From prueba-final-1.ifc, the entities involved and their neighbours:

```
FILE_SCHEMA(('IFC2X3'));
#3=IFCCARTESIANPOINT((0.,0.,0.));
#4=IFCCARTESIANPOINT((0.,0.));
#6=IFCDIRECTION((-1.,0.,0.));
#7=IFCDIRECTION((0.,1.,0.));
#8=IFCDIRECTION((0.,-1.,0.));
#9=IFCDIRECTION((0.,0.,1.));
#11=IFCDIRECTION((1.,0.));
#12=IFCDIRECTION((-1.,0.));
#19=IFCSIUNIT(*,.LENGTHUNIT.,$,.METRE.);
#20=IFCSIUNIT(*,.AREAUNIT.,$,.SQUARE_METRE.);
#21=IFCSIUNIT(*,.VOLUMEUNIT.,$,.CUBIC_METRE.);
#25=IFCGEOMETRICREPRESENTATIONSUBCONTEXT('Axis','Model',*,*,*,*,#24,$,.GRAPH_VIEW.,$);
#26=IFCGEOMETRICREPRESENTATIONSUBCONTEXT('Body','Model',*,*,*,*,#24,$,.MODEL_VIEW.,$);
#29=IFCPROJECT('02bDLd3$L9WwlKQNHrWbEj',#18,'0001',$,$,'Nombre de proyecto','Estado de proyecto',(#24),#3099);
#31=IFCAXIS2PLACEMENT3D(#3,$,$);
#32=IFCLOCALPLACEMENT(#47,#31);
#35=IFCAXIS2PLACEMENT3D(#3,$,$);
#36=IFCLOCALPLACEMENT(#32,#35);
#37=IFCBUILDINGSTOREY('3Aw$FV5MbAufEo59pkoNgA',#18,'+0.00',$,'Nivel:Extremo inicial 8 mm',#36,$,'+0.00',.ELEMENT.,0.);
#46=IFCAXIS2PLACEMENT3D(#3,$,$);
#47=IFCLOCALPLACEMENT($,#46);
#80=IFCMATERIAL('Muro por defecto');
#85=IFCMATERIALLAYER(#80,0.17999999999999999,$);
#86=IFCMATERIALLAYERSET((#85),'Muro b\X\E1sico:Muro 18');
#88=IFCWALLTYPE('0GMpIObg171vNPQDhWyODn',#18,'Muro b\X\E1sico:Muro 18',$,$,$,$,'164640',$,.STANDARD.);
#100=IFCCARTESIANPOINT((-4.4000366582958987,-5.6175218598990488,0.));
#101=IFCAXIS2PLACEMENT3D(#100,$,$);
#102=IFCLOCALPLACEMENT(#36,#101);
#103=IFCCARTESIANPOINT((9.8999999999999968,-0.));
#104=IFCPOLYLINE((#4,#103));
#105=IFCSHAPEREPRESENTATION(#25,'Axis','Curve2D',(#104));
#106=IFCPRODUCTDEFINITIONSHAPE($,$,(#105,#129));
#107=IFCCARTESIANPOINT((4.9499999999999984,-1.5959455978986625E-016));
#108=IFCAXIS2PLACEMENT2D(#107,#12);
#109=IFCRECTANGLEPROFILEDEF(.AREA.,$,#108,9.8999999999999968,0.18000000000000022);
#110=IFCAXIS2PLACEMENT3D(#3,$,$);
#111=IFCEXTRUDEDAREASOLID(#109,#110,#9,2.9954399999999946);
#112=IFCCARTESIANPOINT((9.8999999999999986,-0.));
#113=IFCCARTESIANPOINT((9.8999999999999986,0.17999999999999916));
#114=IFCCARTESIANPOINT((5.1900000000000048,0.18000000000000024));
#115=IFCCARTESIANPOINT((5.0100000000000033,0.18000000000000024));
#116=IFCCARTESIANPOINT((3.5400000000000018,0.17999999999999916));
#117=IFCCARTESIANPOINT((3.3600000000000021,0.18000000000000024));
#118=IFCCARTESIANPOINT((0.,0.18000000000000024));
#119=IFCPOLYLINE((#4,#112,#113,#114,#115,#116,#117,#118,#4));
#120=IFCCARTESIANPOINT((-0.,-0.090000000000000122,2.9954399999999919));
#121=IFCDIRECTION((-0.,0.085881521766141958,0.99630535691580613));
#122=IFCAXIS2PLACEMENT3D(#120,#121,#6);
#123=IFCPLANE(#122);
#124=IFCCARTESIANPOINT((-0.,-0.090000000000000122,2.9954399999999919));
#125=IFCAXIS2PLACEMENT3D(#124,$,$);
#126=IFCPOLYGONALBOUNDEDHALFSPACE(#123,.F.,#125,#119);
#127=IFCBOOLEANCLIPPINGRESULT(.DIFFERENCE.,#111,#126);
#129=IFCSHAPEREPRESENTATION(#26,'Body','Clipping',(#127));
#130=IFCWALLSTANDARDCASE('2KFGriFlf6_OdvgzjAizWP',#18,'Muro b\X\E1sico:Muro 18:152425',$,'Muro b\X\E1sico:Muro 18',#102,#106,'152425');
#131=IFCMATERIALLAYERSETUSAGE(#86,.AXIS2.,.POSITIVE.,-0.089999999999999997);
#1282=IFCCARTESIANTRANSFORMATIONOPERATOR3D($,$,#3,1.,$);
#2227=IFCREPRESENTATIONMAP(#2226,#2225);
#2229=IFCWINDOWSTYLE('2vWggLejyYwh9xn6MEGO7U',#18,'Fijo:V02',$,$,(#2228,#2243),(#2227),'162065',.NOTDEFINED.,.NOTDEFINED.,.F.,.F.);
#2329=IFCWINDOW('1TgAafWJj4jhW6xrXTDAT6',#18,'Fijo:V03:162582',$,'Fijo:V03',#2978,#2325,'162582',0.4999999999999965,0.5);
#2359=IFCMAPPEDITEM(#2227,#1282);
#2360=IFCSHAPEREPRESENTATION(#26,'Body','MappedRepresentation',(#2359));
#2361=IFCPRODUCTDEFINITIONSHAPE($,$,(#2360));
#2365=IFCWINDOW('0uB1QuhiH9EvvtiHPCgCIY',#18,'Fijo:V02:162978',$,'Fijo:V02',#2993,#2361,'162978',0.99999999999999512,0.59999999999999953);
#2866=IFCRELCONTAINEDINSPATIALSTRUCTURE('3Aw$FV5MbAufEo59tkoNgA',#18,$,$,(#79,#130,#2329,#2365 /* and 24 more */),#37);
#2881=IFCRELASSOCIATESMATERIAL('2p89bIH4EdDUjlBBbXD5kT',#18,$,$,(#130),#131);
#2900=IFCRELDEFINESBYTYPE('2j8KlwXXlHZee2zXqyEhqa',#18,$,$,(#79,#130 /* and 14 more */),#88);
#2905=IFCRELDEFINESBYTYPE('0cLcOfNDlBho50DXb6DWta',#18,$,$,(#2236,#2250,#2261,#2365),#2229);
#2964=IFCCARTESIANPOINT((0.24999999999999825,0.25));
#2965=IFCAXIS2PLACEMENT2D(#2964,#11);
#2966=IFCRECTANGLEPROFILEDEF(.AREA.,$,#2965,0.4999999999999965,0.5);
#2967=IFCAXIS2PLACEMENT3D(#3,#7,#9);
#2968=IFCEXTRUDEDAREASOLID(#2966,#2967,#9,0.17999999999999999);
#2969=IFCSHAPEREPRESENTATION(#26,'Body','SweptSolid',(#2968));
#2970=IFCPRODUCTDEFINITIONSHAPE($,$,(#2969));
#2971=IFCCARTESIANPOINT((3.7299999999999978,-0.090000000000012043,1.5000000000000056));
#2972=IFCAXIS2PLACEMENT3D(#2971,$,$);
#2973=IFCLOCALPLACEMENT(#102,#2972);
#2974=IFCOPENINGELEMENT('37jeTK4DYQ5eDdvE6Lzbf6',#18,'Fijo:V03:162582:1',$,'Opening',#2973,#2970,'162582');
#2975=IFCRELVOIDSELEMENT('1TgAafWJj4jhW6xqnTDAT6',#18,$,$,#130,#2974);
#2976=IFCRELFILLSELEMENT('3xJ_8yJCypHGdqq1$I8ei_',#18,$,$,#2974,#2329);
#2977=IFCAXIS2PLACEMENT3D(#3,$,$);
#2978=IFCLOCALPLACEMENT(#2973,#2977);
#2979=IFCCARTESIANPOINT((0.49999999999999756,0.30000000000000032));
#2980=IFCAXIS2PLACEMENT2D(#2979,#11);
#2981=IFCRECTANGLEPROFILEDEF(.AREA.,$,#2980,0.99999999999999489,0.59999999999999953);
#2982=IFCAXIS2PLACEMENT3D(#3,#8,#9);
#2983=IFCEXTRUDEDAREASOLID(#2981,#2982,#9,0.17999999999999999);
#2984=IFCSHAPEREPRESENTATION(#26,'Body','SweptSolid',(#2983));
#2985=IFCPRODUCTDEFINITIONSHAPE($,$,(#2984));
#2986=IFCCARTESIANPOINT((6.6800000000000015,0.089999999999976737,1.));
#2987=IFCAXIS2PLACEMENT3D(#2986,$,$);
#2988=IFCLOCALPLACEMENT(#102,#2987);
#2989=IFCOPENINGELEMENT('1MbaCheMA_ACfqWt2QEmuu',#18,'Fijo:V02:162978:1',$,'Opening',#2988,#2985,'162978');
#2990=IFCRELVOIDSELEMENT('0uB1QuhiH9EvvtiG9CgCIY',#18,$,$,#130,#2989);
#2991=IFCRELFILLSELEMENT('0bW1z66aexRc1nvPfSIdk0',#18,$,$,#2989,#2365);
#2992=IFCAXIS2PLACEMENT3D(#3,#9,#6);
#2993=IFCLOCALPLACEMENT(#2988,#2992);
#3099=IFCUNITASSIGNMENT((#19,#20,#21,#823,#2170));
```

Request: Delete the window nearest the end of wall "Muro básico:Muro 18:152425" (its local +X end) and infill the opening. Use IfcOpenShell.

```python
import ifcopenshell
import ifcopenshell.api.feature
import ifcopenshell.api.root
import ifcopenshell.geom
import ifcopenshell.util.shape

model = ifcopenshell.open("prueba-final-1.ifc")
settings = ifcopenshell.geom.settings()


def volume(element):
    """Net volume in cubic metres, openings subtracted."""
    shape = ifcopenshell.geom.create_shape(settings, element)
    return ifcopenshell.util.shape.get_volume(shape.geometry)


window = model.by_guid("0uB1QuhiH9EvvtiHPCgCIY")
opening = window.FillsVoids[0].RelatingOpeningElement
wall = opening.VoidsElements[0].RelatingBuildingElement
before = volume(wall)

ifcopenshell.api.root.remove_product(model, product=window)
ifcopenshell.api.feature.remove_feature(model, feature=opening)

after = volume(wall)

print(f"wall volume {before:.3f} -> {after:.3f} m3")

model.write("prueba-final-1_edited.ifc")
```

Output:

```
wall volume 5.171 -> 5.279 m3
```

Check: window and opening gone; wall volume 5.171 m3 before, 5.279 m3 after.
